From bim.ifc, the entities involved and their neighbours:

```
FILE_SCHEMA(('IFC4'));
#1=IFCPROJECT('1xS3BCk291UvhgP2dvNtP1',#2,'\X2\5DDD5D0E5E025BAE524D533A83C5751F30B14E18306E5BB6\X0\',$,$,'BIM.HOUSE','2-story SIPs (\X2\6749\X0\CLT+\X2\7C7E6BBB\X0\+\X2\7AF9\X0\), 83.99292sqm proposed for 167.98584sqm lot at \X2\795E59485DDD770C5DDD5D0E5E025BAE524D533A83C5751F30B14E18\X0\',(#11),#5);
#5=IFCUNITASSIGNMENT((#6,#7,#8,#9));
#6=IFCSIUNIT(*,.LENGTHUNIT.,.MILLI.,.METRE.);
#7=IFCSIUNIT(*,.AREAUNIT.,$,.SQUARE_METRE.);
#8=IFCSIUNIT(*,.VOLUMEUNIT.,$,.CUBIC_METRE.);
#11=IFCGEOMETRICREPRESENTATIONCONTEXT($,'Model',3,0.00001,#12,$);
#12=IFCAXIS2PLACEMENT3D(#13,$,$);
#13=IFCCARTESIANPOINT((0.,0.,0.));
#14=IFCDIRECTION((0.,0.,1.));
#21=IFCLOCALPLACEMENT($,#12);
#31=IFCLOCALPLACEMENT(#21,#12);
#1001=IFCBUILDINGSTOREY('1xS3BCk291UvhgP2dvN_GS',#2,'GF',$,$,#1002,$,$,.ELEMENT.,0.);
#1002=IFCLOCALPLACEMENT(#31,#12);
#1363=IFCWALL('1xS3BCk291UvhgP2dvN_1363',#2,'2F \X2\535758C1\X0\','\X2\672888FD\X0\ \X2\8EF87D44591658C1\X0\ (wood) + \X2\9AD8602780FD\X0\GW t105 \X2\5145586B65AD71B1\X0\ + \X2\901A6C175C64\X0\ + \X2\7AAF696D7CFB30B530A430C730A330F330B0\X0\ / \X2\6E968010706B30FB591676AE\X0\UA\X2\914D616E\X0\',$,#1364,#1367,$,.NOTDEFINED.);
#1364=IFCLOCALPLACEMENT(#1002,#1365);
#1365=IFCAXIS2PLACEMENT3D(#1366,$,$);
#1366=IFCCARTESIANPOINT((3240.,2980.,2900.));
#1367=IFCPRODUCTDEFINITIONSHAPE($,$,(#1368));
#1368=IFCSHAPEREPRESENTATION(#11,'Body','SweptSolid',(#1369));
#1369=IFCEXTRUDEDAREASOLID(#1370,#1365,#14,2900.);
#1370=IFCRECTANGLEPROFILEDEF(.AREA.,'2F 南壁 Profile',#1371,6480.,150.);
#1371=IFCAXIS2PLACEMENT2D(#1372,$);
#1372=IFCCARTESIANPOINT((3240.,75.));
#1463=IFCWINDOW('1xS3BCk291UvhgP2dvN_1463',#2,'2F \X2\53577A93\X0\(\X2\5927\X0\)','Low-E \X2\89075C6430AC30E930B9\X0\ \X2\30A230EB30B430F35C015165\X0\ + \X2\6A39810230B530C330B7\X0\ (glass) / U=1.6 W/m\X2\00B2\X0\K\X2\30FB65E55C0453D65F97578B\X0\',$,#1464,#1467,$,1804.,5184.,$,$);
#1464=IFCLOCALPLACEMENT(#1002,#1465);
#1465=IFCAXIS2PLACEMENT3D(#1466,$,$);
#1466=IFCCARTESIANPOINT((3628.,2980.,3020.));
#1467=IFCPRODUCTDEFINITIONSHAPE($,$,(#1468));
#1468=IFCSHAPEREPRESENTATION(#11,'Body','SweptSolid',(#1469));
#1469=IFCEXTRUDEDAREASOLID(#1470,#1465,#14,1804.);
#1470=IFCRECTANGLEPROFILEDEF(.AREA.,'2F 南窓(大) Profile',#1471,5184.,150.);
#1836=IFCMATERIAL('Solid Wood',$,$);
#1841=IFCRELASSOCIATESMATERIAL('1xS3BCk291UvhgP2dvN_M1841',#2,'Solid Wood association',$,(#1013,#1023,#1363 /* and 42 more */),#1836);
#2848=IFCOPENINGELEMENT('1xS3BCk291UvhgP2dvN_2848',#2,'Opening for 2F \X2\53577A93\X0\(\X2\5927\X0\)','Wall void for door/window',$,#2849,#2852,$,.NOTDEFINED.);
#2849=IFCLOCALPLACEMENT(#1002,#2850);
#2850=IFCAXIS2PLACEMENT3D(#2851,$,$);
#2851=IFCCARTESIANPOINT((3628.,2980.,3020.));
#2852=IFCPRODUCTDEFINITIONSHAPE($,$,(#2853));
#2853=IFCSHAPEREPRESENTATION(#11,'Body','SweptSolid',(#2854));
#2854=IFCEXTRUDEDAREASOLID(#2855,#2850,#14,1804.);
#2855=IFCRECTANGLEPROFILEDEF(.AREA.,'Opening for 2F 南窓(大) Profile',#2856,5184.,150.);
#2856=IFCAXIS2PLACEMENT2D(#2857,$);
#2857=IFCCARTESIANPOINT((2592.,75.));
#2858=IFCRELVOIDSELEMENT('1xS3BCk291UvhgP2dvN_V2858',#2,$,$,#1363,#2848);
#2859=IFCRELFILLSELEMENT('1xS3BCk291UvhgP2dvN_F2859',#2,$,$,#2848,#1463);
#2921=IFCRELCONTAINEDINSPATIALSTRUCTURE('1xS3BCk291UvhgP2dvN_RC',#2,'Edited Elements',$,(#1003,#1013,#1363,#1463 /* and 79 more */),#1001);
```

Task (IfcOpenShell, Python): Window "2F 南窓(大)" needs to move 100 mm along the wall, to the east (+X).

```python
import ifcopenshell
import ifcopenshell.api.geometry
import ifcopenshell.util.placement

model = ifcopenshell.open("bim.ifc")

window = model.by_id(1463)
opening = window.FillsVoids[0].RelatingOpeningElement
wall = opening.VoidsElements[0].RelatingBuildingElement

wall_matrix = ifcopenshell.util.placement.get_local_placement(wall.ObjectPlacement)
shift = wall_matrix[:3, 0] * 100.0
before = ifcopenshell.util.placement.get_local_placement(window.ObjectPlacement)[:3, 3].copy()

# The window is not placed relative to its opening, so move both.
for product in (opening, window):
    matrix = ifcopenshell.util.placement.get_local_placement(product.ObjectPlacement)
    matrix[:3, 3] += shift
    ifcopenshell.api.geometry.edit_object_placement(model, product=product, matrix=matrix, is_si=False)

after = ifcopenshell.util.placement.get_local_placement(window.ObjectPlacement)[:3, 3]
print("window moved by", (after - before).round(3) + 0.0)

model.write("bim-out.ifc")
```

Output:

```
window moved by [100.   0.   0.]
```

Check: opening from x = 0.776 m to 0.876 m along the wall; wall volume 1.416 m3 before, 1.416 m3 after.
